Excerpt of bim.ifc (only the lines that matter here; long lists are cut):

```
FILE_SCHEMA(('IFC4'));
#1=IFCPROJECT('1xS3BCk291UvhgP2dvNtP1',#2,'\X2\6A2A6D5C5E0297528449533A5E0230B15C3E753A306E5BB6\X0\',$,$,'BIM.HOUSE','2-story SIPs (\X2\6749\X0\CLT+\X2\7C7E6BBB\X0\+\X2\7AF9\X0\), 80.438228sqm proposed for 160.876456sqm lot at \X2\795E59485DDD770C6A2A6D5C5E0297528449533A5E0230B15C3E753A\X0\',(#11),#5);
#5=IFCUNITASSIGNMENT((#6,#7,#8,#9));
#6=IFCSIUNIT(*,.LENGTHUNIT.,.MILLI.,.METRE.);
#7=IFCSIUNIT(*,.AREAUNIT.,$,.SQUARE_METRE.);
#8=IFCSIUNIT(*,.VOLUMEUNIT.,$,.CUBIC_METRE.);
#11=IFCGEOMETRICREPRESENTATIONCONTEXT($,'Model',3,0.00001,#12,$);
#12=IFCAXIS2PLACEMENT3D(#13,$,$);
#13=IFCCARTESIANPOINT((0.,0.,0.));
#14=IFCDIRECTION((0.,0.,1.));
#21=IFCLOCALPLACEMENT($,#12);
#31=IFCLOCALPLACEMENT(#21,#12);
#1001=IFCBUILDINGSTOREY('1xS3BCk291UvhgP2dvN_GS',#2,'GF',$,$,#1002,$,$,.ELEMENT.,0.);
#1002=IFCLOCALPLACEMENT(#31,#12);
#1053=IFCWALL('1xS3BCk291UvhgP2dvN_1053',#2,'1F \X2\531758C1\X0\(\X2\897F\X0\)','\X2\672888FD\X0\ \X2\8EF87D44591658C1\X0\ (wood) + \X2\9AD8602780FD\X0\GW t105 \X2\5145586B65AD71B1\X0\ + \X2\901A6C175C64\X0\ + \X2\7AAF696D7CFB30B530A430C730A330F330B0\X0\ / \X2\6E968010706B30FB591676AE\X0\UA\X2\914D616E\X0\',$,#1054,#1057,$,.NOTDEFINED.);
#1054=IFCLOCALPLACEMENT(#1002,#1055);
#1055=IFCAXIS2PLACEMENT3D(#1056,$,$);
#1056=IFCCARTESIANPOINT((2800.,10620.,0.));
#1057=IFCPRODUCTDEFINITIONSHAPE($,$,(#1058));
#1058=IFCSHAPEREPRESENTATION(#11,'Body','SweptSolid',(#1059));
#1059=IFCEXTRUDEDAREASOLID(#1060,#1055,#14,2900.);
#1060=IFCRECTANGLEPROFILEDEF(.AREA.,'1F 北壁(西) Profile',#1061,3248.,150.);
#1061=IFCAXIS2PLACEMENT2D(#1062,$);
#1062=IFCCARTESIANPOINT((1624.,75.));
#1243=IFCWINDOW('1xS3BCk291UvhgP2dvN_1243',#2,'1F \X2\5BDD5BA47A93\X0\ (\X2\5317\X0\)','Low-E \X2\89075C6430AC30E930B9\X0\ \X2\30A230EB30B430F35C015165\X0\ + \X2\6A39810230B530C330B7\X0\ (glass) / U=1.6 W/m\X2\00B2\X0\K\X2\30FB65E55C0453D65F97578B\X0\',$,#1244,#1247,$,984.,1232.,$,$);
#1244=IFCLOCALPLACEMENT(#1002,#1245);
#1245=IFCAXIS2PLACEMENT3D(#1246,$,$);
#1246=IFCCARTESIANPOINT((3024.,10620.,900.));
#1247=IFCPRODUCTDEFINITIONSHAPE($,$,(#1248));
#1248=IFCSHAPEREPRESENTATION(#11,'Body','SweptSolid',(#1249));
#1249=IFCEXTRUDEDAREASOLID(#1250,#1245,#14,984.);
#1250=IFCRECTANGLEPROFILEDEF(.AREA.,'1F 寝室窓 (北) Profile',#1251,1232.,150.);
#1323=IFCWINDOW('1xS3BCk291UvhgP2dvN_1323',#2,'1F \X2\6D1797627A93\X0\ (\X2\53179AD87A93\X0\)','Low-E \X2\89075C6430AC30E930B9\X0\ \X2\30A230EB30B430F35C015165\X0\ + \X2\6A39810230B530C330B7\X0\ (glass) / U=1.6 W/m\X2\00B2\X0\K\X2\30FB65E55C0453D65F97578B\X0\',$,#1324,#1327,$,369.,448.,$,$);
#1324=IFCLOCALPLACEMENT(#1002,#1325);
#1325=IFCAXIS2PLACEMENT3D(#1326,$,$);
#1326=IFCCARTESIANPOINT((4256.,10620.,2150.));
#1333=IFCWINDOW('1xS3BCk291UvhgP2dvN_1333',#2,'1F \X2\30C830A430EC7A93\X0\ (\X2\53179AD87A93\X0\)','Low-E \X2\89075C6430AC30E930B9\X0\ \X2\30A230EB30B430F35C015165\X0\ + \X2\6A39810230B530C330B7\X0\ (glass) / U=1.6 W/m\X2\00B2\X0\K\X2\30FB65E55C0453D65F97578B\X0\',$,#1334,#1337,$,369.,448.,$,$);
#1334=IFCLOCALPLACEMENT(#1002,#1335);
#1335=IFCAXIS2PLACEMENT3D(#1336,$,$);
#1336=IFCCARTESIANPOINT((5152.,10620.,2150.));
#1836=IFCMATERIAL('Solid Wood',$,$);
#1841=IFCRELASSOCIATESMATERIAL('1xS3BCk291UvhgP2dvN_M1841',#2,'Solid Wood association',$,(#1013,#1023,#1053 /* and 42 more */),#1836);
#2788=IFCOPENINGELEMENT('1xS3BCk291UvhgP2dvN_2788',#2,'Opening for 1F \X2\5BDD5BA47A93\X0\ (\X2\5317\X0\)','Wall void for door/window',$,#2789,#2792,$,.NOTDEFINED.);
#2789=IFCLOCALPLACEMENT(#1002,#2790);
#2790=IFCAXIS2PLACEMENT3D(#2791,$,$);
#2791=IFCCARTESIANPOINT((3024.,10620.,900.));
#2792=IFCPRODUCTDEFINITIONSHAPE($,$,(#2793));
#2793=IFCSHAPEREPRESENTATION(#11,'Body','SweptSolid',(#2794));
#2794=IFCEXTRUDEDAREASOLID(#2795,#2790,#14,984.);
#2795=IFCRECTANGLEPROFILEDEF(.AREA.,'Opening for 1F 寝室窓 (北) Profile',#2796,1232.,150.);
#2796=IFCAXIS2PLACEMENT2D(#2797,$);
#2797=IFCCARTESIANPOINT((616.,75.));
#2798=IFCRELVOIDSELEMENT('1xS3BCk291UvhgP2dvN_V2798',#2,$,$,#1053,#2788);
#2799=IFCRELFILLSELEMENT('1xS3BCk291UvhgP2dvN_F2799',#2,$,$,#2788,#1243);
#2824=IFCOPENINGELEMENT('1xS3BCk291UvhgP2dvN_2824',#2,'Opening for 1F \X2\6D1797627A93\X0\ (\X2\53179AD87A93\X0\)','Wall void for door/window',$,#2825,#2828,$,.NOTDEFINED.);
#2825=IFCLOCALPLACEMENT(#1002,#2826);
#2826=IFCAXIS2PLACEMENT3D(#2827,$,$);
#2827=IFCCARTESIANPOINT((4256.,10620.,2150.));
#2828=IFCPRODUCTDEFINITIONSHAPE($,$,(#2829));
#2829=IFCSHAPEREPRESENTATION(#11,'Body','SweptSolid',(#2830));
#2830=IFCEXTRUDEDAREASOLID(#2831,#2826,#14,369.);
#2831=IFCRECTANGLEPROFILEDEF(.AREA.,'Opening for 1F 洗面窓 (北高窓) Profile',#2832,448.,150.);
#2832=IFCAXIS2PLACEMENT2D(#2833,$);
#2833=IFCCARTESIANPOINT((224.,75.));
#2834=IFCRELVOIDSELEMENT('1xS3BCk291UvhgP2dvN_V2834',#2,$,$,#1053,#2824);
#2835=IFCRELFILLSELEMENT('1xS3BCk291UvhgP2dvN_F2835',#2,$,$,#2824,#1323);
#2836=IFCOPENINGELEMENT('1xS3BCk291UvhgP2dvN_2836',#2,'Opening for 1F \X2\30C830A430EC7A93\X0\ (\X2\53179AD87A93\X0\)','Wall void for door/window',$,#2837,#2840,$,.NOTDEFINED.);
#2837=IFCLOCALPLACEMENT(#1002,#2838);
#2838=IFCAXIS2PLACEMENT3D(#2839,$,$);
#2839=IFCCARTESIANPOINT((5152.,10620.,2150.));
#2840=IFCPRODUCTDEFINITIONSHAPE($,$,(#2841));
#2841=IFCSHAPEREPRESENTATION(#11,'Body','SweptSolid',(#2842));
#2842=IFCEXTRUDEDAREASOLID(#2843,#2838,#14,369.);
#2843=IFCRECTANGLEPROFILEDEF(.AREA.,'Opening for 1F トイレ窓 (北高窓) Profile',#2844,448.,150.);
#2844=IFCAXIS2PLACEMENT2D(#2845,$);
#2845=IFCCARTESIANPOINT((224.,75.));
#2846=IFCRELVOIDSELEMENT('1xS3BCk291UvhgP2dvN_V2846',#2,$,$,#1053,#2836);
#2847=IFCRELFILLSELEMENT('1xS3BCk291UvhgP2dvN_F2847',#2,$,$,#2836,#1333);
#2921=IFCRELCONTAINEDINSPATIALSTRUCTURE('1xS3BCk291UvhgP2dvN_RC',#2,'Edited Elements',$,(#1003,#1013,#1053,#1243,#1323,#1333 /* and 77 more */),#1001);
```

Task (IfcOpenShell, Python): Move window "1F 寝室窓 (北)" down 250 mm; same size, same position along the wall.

```python
import numpy as np
import ifcopenshell
import ifcopenshell.api.geometry
import ifcopenshell.util.placement
import ifcopenshell.util.unit

model = ifcopenshell.open("bim.ifc")
unit_scale = ifcopenshell.util.unit.calculate_unit_scale(model)

window = model.by_id(1243)
opening = window.FillsVoids[0].RelatingOpeningElement
dz = -0.25 / unit_scale

shift = np.array([0.0, 0.0, dz])
# The window is not placed relative to its opening, so move both.
for product in (opening, window):
    matrix = ifcopenshell.util.placement.get_local_placement(product.ObjectPlacement)
    matrix[:3, 3] += shift
    ifcopenshell.api.geometry.edit_object_placement(model, product=product, matrix=matrix, is_si=False)

print(f"moved by {dz * unit_scale:+.3f} m")

model.write("bim_edited.ifc")
```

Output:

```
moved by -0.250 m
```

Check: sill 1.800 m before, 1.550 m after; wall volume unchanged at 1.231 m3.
